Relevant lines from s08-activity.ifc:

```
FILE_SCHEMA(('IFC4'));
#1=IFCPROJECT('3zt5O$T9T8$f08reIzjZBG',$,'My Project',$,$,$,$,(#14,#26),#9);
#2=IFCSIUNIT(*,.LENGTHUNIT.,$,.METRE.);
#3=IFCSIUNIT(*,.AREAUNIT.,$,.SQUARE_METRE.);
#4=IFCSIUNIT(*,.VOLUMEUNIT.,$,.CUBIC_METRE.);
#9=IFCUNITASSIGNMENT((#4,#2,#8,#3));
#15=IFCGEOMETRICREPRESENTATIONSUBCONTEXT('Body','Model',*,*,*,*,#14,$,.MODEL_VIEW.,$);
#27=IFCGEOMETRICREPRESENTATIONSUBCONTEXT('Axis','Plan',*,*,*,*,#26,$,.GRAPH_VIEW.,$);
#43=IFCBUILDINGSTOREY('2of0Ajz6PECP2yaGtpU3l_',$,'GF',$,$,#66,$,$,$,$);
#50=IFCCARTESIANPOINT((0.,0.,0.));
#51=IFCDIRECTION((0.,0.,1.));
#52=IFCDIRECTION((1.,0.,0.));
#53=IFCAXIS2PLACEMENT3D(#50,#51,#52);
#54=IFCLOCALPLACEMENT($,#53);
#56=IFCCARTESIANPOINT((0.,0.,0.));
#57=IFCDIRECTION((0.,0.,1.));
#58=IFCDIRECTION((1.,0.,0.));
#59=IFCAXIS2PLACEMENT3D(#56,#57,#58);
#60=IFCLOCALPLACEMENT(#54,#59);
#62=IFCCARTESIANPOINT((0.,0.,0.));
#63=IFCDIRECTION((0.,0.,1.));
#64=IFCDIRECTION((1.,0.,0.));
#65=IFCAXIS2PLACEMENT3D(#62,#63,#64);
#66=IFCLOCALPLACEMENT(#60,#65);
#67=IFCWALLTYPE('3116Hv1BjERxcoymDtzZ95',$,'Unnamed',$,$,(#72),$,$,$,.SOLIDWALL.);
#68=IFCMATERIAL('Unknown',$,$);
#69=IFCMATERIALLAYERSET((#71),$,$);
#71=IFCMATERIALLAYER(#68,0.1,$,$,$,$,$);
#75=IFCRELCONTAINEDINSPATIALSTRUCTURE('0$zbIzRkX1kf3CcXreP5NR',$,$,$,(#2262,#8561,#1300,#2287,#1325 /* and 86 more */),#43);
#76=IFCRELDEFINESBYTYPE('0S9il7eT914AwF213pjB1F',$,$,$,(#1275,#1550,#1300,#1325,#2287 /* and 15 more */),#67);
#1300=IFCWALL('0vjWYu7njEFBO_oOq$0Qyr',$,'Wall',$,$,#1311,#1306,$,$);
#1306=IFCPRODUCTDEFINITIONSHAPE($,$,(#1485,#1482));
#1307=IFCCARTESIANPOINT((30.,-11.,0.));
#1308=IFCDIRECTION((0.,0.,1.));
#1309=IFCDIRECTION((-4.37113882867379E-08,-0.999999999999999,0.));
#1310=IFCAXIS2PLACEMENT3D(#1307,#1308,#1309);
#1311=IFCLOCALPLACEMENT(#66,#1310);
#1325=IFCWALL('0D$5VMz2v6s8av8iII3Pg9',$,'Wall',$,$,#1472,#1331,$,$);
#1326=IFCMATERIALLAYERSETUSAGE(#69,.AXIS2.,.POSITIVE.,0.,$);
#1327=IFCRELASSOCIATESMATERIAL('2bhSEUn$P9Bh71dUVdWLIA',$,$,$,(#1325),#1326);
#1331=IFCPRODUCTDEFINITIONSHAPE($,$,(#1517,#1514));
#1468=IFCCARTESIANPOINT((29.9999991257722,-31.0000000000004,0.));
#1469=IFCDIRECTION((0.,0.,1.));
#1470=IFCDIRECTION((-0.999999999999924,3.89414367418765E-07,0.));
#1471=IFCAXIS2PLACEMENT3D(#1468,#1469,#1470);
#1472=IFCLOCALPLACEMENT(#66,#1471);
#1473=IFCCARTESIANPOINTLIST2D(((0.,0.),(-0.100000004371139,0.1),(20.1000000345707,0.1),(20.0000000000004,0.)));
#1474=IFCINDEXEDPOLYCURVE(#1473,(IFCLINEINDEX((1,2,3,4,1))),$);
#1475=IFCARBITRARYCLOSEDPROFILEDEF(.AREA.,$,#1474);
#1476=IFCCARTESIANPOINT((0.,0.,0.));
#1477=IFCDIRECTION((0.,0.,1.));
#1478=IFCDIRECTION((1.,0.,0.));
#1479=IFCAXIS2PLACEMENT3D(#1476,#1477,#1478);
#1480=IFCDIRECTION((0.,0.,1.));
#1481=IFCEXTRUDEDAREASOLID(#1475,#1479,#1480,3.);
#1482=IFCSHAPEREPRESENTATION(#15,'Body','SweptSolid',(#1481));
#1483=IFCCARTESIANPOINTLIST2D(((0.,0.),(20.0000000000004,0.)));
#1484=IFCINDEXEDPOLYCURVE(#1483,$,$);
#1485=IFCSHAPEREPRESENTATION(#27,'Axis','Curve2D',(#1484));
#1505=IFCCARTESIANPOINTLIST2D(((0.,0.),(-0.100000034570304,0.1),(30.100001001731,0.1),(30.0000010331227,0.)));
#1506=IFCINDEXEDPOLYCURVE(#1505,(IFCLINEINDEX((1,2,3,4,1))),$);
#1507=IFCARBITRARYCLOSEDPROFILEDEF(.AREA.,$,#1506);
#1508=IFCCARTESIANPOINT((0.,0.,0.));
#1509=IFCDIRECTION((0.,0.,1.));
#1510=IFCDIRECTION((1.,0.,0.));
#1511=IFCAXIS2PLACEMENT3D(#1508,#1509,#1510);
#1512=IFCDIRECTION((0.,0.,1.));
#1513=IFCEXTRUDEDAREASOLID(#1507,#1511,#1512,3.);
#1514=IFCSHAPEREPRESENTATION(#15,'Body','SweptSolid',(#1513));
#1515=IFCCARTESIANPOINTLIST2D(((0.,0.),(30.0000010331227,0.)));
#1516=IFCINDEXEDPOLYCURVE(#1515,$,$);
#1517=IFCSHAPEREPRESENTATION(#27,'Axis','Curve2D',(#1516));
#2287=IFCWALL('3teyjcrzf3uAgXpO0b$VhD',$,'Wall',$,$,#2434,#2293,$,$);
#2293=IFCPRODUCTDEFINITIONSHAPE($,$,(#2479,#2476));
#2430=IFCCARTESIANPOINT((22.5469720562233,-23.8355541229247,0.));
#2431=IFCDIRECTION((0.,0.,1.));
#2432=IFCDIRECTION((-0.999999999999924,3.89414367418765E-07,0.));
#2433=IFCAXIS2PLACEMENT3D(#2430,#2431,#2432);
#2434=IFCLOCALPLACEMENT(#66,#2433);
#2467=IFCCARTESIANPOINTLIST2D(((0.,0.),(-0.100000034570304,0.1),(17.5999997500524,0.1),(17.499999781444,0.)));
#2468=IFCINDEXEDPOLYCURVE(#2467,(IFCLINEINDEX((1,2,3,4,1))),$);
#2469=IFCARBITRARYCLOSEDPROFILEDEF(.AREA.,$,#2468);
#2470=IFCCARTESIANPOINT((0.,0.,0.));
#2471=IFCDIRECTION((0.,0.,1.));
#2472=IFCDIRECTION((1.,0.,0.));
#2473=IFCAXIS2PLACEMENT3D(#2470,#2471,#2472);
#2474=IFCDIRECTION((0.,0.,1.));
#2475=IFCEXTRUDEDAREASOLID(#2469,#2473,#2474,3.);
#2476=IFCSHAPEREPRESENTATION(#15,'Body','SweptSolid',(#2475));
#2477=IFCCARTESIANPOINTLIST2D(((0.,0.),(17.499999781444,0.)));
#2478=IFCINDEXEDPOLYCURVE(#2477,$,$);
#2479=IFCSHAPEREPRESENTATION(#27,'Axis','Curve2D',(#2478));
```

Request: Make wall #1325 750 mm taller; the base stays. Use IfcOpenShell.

```python
import ifcopenshell
import ifcopenshell.geom
import ifcopenshell.util.representation
import ifcopenshell.util.shape

model = ifcopenshell.open("s08-activity.ifc")
settings = ifcopenshell.geom.settings()


def volume(element):
    """Net volume in cubic metres, openings subtracted."""
    shape = ifcopenshell.geom.create_shape(settings, element)
    return ifcopenshell.util.shape.get_volume(shape.geometry)


wall = model.by_guid("0D$5VMz2v6s8av8iII3Pg9")
before = volume(wall)

body = ifcopenshell.util.representation.get_representation(wall, "Model", "Body")
solid = body.Items[0]
old_height = solid.Depth
solid.Depth += 0.75
after = volume(wall)

print(f"height {old_height:g} -> {solid.Depth:g}, volume {before:.3f} -> {after:.3f} m3")

model.write("s08-activity_rev.ifc")
```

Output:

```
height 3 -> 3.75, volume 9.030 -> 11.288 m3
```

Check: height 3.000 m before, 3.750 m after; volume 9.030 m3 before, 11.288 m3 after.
